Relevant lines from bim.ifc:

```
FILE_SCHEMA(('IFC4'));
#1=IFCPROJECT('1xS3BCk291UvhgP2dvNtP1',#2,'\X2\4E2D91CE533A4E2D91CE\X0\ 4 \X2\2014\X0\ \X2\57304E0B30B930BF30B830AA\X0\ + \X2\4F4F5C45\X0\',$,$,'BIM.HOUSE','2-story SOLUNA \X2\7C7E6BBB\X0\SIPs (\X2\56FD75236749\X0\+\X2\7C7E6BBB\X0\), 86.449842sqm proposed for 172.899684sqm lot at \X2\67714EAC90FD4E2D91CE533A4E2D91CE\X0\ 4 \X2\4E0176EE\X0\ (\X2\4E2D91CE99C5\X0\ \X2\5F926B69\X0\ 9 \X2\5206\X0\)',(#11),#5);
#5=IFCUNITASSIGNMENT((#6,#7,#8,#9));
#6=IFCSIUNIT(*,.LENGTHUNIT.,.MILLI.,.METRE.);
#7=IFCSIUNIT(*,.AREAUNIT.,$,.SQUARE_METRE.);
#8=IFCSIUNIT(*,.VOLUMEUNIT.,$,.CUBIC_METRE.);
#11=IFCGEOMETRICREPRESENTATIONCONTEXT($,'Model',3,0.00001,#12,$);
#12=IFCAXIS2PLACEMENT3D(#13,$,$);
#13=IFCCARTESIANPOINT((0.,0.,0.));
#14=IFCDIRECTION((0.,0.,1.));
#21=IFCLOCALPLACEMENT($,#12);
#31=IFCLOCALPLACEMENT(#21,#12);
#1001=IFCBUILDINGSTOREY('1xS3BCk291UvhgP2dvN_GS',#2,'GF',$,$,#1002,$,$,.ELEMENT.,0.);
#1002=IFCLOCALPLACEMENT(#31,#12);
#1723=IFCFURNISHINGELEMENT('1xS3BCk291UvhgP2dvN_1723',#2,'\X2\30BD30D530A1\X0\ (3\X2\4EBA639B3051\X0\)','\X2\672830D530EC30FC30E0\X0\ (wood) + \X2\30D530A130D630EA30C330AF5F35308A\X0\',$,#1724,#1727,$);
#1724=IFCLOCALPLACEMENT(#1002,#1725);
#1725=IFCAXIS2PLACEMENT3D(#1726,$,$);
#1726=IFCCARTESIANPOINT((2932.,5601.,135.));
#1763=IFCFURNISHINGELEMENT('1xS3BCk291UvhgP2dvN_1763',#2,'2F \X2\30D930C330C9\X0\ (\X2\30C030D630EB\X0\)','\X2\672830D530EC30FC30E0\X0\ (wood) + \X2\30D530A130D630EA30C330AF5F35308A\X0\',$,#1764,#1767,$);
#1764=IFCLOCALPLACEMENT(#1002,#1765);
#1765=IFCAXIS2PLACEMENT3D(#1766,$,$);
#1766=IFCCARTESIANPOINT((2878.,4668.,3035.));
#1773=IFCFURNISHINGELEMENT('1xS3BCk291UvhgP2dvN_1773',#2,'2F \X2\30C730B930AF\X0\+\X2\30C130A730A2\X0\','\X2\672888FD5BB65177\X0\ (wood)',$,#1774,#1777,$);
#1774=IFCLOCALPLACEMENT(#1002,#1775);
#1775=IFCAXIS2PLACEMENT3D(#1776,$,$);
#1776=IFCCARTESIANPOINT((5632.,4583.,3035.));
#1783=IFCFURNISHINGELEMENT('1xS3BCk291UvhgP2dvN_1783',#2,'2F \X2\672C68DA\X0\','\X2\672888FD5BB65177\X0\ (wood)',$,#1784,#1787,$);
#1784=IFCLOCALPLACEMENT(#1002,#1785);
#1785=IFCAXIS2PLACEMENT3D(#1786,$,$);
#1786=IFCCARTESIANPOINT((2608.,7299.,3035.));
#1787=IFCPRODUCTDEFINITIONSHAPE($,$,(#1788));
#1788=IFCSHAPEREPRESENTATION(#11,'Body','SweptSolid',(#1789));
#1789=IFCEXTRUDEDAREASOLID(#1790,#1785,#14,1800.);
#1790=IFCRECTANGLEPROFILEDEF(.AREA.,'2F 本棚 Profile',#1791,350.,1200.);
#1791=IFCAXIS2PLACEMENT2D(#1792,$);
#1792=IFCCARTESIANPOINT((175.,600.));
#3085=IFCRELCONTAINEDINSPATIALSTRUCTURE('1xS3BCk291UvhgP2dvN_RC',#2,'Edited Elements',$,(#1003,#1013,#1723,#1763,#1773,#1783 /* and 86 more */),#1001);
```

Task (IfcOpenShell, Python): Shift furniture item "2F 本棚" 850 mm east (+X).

```python
import ifcopenshell
import ifcopenshell.api.geometry
import ifcopenshell.util.placement
import ifcopenshell.util.unit

model = ifcopenshell.open("bim.ifc")
unit_scale = ifcopenshell.util.unit.calculate_unit_scale(model)

item = model.by_id(1783)
matrix = ifcopenshell.util.placement.get_local_placement(item.ObjectPlacement)
matrix[0, 3] += 0.85 / unit_scale
ifcopenshell.api.geometry.edit_object_placement(model, product=item, matrix=matrix, is_si=False)

print(ifcopenshell.util.placement.get_local_placement(item.ObjectPlacement).round(3) + 0.0)

model.write("bim_rev.ifc")
```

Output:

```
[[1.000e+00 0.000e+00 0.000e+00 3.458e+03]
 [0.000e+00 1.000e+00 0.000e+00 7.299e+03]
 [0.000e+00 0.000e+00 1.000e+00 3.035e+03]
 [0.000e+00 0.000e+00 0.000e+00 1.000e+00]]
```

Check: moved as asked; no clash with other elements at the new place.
